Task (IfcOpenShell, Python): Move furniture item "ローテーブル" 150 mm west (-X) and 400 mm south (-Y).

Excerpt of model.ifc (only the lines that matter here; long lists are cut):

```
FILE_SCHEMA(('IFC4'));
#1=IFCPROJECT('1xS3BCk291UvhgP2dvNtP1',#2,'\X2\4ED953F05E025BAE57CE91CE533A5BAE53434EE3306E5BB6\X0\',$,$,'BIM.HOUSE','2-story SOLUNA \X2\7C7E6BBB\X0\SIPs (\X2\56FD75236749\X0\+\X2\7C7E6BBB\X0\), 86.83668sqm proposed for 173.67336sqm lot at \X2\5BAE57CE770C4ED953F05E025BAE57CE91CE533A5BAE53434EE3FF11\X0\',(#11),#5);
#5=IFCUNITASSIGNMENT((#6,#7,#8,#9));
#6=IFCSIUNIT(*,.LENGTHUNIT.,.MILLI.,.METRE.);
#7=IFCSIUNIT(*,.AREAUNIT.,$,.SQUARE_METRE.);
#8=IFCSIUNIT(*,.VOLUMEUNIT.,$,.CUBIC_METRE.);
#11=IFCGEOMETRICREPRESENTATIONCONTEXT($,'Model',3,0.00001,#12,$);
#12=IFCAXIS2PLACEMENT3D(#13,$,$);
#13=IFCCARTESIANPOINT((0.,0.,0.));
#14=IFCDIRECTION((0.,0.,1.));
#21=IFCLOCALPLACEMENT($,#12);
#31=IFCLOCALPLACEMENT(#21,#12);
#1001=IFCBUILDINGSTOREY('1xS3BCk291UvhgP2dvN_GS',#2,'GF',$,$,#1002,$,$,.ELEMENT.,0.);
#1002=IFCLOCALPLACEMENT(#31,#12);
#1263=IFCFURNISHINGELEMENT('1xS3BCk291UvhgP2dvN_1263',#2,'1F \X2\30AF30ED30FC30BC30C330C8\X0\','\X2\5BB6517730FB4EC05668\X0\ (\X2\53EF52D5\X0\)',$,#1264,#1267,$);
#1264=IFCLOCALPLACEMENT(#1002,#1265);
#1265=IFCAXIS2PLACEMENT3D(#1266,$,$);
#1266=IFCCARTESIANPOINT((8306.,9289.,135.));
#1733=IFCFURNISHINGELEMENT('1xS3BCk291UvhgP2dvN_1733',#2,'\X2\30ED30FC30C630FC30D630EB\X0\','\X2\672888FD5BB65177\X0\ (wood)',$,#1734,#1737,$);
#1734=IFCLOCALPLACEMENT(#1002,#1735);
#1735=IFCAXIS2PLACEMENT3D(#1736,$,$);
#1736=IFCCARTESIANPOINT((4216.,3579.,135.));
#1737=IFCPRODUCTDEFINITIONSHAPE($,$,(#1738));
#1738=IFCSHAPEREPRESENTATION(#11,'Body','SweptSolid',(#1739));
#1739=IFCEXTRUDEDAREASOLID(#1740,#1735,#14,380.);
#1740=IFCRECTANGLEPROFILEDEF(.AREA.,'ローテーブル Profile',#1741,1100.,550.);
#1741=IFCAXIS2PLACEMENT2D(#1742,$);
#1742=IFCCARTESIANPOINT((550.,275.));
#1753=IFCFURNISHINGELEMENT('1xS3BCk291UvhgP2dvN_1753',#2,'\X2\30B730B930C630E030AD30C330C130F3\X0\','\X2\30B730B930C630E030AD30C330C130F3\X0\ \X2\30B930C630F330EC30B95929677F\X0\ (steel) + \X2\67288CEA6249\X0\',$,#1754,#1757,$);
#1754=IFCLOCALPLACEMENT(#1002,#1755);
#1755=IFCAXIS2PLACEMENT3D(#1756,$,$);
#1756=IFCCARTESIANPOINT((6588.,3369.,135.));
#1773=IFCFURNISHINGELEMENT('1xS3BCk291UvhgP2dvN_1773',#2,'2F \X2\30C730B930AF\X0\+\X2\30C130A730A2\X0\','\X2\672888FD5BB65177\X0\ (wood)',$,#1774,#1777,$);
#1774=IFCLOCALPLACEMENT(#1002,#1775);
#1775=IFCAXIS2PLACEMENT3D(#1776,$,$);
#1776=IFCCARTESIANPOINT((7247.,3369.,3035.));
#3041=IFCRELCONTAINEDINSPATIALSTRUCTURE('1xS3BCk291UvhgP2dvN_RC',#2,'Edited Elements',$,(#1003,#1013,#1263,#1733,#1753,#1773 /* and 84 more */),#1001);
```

```python
import ifcopenshell
import ifcopenshell.api.geometry
import ifcopenshell.util.placement
import ifcopenshell.util.unit

model = ifcopenshell.open("model.ifc")
unit_scale = ifcopenshell.util.unit.calculate_unit_scale(model)

item = model.by_guid("1xS3BCk291UvhgP2dvN_1733")
matrix = ifcopenshell.util.placement.get_local_placement(item.ObjectPlacement)
matrix[0, 3] -= 0.15 / unit_scale
matrix[1, 3] -= 0.4 / unit_scale
ifcopenshell.api.geometry.edit_object_placement(model, product=item, matrix=matrix, is_si=False)

print(ifcopenshell.util.placement.get_local_placement(item.ObjectPlacement).round(3) + 0.0)

model.write("model_v2.ifc")
```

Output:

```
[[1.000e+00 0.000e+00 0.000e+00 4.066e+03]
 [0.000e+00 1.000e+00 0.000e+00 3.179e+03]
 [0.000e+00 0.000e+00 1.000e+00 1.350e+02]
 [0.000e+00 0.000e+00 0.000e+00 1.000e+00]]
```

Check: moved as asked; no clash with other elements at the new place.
